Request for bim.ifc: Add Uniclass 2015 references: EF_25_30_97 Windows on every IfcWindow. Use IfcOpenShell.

First a look at what the model holds.

```python
import ifcopenshell

model = ifcopenshell.open("bim.ifc")
print(model.schema)
print("classifications:", [c.Name for c in model.by_type("IfcClassification")])
for ifc_class in ("IfcDoor", "IfcRoof", "IfcStair", "IfcWall", "IfcWindow"):
    print(ifc_class, len(model.by_type(ifc_class)))
```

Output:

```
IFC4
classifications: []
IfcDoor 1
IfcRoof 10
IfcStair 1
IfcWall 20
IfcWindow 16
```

```python
import ifcopenshell
import ifcopenshell.api.classification

model = ifcopenshell.open("bim.ifc")

system = ifcopenshell.api.classification.add_classification(model, classification="Uniclass 2015")

codes = {
    "IfcWindow": ("EF_25_30_97", "Windows"),
}
for ifc_class, (code, name) in codes.items():
    products = model.by_type(ifc_class)
    ifcopenshell.api.classification.add_reference(
        model, products=products, classification=system, identification=code, name=name
    )
    print(code, len(products))

model.write("bim_v2.ifc")
```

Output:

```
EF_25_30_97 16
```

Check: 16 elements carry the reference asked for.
